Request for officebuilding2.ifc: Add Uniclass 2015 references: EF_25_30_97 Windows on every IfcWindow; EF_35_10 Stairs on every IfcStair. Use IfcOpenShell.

First a look at what the model holds.

```python
import ifcopenshell

model = ifcopenshell.open("officebuilding2.ifc")
print(model.schema)
print("classifications:", [c.Name for c in model.by_type("IfcClassification")])
for ifc_class in ("IfcDoor", "IfcRoof", "IfcStair", "IfcWall", "IfcWindow"):
    print(ifc_class, len(model.by_type(ifc_class)))
```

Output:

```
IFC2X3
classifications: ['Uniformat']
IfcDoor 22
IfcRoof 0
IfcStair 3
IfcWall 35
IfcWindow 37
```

```python
import ifcopenshell
import ifcopenshell.api.classification

model = ifcopenshell.open("officebuilding2.ifc")

# IFC2X3 requires Source and Edition and has no link from the project to the system.
system = model.create_entity("IfcClassification", Source="NBS", Edition="2015", Name="Uniclass 2015")

codes = {
    "IfcWindow": ("EF_25_30_97", "Windows"),
    "IfcStair": ("EF_35_10", "Stairs"),
}
for ifc_class, (code, name) in codes.items():
    products = model.by_type(ifc_class)
    ifcopenshell.api.classification.add_reference(
        model, products=products, classification=system, identification=code, name=name
    )
    print(code, len(products))

model.write("officebuilding2_updated.ifc")
```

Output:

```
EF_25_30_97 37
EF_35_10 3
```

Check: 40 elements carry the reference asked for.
